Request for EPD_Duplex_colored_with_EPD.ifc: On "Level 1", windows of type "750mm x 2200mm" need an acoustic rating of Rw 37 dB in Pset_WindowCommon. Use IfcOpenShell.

First a look at what the model holds.

```python
import ifcopenshell
import ifcopenshell.util.element

model = ifcopenshell.open("EPD_Duplex_colored_with_EPD.ifc")
print(model.schema)
storey = next(s for s in model.by_type("IfcBuildingStorey") if s.Name == "Level 1")
windows = [e for e in ifcopenshell.util.element.get_decomposition(storey) if e.is_a("IfcWindow")]
seen = {}
for e in windows:
    element_type = ifcopenshell.util.element.get_type(e)
    key = (element_type.Name if element_type != e and element_type else None, ifcopenshell.util.element.get_pset(e, "Pset_WindowCommon", "AcousticRating"))
    seen[key] = seen.get(key, 0) + 1
for (name, value), count in sorted(seen.items(), key=str):
    print(count, "x", name, "|", value)
```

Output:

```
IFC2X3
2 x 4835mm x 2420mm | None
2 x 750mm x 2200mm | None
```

```python
import ifcopenshell
import ifcopenshell.api.pset
import ifcopenshell.util.element

model = ifcopenshell.open("EPD_Duplex_colored_with_EPD.ifc")

storey = next(s for s in model.by_type("IfcBuildingStorey") if s.Name == "Level 1")
windows = [e for e in ifcopenshell.util.element.get_decomposition(storey) if e.is_a("IfcWindow")]

count = 0
for e in windows:
    element_type = ifcopenshell.util.element.get_type(e)
    if element_type in (None, e) or element_type.Name != "750mm x 2200mm":
        continue
    # add_pset returns the element's existing set when there is one.
    pset = ifcopenshell.api.pset.add_pset(model, product=e, name="Pset_WindowCommon")
    ifcopenshell.api.pset.edit_pset(model, pset=pset, properties={"AcousticRating": "Rw 37 dB"})
    count += 1

print(count, "windows updated")

model.write("EPD_Duplex_colored_with_EPD-out.ifc")
```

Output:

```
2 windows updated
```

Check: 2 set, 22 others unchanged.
